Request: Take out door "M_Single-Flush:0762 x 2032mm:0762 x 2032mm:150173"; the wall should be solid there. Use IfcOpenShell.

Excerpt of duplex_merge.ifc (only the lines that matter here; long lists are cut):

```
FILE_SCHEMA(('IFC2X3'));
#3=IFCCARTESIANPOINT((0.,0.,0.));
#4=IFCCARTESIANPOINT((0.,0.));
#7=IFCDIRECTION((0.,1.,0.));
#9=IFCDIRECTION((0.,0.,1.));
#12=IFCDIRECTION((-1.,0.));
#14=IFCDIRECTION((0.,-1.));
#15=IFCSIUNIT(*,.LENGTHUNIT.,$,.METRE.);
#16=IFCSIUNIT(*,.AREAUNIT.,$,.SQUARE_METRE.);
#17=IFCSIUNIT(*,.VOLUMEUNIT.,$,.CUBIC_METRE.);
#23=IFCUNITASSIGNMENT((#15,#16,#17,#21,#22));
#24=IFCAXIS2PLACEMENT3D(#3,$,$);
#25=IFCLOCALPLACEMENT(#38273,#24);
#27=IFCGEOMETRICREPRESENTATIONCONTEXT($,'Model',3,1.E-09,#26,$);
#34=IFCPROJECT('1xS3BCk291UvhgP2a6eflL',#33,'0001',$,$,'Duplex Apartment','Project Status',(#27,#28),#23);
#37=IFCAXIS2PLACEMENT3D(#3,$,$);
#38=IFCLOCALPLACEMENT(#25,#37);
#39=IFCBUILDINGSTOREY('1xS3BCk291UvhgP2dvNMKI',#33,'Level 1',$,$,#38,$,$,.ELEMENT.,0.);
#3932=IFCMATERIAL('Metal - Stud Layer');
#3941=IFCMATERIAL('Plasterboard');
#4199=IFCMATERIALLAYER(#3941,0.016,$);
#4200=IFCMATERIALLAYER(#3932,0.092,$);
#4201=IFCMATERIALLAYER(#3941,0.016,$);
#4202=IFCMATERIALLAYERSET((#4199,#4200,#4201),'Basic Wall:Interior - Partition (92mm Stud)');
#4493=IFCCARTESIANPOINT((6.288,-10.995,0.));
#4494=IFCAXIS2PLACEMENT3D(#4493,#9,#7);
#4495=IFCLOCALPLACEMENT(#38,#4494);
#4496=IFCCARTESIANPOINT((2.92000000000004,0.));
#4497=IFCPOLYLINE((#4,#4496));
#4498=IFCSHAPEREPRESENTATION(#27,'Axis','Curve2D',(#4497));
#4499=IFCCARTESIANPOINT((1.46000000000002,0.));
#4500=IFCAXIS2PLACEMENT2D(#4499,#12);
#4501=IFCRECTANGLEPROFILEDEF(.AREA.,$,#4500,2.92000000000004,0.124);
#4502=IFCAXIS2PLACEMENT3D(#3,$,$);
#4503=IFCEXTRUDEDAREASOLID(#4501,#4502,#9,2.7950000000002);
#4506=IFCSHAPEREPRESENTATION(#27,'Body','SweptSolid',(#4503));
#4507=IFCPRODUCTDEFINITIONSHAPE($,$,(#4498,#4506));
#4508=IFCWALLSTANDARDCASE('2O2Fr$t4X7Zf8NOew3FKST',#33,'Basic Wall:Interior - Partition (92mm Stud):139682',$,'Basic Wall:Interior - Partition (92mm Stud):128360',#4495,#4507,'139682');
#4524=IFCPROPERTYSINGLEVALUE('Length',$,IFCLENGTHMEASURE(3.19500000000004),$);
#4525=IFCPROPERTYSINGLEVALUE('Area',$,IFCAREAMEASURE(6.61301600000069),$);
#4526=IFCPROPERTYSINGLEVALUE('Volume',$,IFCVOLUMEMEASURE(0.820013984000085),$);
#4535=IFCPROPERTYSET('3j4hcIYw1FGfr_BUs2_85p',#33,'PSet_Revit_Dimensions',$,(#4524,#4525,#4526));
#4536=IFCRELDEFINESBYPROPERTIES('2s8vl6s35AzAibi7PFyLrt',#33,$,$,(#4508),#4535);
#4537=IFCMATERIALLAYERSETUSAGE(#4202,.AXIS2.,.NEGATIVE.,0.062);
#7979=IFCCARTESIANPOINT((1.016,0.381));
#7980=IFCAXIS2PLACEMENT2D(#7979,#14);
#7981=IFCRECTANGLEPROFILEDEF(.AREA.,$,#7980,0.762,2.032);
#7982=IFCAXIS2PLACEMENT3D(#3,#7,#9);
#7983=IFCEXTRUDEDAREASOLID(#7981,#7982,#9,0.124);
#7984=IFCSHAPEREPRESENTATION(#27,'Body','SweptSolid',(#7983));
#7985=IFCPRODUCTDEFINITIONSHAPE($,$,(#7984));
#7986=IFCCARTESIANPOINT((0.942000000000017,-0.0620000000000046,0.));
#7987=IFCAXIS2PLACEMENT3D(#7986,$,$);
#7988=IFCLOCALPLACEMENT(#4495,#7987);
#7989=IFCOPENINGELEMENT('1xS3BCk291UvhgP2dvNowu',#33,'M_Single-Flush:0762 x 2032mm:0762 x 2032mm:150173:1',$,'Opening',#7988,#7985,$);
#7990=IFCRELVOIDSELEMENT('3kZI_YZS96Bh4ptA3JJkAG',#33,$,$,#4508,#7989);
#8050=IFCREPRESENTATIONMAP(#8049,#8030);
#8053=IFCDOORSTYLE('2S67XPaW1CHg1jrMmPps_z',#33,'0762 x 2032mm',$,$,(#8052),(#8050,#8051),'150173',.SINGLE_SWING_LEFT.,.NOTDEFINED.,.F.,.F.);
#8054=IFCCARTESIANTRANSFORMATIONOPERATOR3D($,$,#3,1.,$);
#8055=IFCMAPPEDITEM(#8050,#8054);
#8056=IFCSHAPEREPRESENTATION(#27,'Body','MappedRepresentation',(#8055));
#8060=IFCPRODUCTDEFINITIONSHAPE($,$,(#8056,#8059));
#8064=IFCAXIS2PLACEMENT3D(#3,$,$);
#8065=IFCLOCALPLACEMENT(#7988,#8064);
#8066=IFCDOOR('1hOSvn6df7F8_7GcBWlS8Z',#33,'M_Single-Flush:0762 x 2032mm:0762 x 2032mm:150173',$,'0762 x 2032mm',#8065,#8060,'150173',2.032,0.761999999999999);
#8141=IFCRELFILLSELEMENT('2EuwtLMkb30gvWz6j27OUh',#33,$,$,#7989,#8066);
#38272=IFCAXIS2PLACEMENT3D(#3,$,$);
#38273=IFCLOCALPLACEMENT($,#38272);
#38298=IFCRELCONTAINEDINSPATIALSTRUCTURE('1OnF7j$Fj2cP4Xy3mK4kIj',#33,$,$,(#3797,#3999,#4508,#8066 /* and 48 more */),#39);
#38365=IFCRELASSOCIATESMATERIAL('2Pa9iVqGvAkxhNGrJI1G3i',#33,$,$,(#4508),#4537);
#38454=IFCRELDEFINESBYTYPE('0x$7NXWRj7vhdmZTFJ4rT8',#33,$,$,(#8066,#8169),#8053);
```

```python
import ifcopenshell
import ifcopenshell.api.feature
import ifcopenshell.api.pset
import ifcopenshell.api.root
import ifcopenshell.geom
import ifcopenshell.util.element
import ifcopenshell.util.shape
import ifcopenshell.util.unit

model = ifcopenshell.open("duplex_merge.ifc")
area_scale = ifcopenshell.util.unit.calculate_unit_scale(model, "AREAUNIT")
volume_scale = ifcopenshell.util.unit.calculate_unit_scale(model, "VOLUMEUNIT")
settings = ifcopenshell.geom.settings()


def volume(element):
    """Net volume in cubic metres, openings subtracted."""
    shape = ifcopenshell.geom.create_shape(settings, element)
    return ifcopenshell.util.shape.get_volume(shape.geometry)


door = model.by_id(8066)
opening = door.FillsVoids[0].RelatingOpeningElement
wall = opening.VoidsElements[0].RelatingBuildingElement
before = volume(wall)

ifcopenshell.api.root.remove_product(model, product=door)
ifcopenshell.api.feature.remove_feature(model, feature=opening)

after = volume(wall)
thickness = 0.124  # wall thickness in metres

# Update the wall's stored quantities.
pset = model.by_id(ifcopenshell.util.element.get_pset(wall, "PSet_Revit_Dimensions", should_inherit=False)["id"])
ifcopenshell.api.pset.edit_pset(model, pset=pset, properties={
    "Area": model.create_entity("IfcAreaMeasure", after / thickness / area_scale),
    "Volume": model.create_entity("IfcVolumeMeasure", after / volume_scale),
})

print(f"wall volume {before:.3f} -> {after:.3f} m3")

model.write("duplex_merge_updated.ifc")
```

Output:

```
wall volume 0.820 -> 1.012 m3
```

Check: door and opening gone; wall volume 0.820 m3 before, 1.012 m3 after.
